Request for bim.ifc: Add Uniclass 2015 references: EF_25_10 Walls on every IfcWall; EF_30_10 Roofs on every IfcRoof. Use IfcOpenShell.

First a look at what the model holds.

```python
import ifcopenshell

model = ifcopenshell.open("bim.ifc")
print(model.schema)
print("classifications:", [c.Name for c in model.by_type("IfcClassification")])
for ifc_class in ("IfcDoor", "IfcRoof", "IfcStair", "IfcWall", "IfcWindow"):
    print(ifc_class, len(model.by_type(ifc_class)))
```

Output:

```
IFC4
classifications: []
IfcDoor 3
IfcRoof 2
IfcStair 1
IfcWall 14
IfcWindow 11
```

```python
import ifcopenshell
import ifcopenshell.api.classification

model = ifcopenshell.open("bim.ifc")

system = ifcopenshell.api.classification.add_classification(model, classification="Uniclass 2015")

codes = {
    "IfcWall": ("EF_25_10", "Walls"),
    "IfcRoof": ("EF_30_10", "Roofs"),
}
for ifc_class, (code, name) in codes.items():
    products = model.by_type(ifc_class)
    ifcopenshell.api.classification.add_reference(
        model, products=products, classification=system, identification=code, name=name
    )
    print(code, len(products))

model.write("bim_edited.ifc")
```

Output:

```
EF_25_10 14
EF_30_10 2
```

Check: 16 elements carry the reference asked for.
